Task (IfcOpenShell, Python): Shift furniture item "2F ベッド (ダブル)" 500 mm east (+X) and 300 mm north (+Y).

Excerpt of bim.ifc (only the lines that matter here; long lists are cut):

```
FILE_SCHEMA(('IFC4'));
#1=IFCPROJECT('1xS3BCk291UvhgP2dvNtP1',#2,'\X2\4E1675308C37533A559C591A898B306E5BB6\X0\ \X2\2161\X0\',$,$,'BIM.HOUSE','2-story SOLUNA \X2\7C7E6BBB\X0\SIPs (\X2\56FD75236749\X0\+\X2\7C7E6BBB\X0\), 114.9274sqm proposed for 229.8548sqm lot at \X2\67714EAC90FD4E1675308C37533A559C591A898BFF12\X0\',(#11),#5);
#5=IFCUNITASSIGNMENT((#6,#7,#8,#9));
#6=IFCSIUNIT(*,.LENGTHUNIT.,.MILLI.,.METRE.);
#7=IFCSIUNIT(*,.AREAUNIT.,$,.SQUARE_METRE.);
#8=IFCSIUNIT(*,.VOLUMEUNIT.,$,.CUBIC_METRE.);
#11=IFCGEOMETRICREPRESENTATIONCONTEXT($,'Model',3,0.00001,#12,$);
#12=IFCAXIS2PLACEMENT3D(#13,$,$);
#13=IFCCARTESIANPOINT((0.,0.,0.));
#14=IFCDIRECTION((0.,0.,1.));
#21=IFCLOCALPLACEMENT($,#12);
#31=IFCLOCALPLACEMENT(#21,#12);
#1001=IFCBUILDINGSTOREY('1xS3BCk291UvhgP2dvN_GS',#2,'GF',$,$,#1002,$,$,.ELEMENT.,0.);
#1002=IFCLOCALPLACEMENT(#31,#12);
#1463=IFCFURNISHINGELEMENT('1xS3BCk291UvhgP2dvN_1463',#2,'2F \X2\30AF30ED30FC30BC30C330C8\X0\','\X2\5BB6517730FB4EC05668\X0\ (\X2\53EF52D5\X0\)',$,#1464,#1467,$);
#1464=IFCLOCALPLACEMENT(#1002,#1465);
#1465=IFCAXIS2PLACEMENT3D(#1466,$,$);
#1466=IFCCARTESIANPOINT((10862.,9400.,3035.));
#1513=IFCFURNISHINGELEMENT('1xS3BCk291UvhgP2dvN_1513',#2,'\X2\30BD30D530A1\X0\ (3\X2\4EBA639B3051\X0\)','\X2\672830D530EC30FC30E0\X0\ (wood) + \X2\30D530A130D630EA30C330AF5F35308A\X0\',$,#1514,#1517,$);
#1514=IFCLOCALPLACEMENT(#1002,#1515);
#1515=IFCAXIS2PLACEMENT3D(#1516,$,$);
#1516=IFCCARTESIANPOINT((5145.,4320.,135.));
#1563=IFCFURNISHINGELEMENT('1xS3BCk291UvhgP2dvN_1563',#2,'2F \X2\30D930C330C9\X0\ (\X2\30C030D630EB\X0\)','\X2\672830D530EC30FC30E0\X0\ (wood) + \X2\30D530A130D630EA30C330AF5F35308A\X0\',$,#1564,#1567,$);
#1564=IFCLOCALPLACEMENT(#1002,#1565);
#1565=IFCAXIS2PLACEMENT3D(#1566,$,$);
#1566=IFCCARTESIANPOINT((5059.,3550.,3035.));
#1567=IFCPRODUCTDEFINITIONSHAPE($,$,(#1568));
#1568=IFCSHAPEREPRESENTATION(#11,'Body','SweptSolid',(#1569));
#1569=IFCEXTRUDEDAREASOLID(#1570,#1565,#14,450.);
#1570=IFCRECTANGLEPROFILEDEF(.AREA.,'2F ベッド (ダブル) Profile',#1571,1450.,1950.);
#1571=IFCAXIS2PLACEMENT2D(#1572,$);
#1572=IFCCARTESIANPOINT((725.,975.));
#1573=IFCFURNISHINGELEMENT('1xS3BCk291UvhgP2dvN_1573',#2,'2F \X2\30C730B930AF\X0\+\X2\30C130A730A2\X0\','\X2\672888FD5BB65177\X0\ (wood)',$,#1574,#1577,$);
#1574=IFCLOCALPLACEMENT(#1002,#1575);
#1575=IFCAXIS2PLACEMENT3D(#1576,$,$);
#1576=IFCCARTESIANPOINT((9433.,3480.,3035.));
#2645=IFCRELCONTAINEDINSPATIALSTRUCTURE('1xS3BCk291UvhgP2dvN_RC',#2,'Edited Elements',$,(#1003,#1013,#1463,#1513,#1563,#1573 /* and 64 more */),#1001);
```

```python
import ifcopenshell
import ifcopenshell.api.geometry
import ifcopenshell.util.placement
import ifcopenshell.util.unit

model = ifcopenshell.open("bim.ifc")
unit_scale = ifcopenshell.util.unit.calculate_unit_scale(model)

item = model.by_guid("1xS3BCk291UvhgP2dvN_1563")
matrix = ifcopenshell.util.placement.get_local_placement(item.ObjectPlacement)
matrix[0, 3] += 0.5 / unit_scale
matrix[1, 3] += 0.3 / unit_scale
ifcopenshell.api.geometry.edit_object_placement(model, product=item, matrix=matrix, is_si=False)

print(ifcopenshell.util.placement.get_local_placement(item.ObjectPlacement).round(3) + 0.0)

model.write("bim_rev.ifc")
```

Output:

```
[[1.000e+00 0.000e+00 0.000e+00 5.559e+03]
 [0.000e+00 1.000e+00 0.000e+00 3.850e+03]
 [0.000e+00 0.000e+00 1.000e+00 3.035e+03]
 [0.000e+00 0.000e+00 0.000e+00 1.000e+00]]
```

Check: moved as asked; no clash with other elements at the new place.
